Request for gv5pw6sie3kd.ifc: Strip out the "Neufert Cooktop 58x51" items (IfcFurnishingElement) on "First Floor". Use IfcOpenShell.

First a look at what the model holds.

```python
import ifcopenshell
import ifcopenshell.util.element

model = ifcopenshell.open("gv5pw6sie3kd.ifc")
print(model.schema)
storey = next(s for s in model.by_type("IfcBuildingStorey") if s.Name == "First Floor")
furniture = [e for e in ifcopenshell.util.element.get_decomposition(storey) if e.is_a("IfcFurnishingElement")]
seen = {}
for e in furniture:
    element_type = ifcopenshell.util.element.get_type(e)
    name = element_type.Name if element_type not in (None, e) else None
    seen[name] = seen.get(name, 0) + 1
for name, count in sorted(seen.items(), key=str):
    print(count, "x", name)
```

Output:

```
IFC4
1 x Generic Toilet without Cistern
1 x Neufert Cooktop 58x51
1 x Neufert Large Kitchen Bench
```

```python
import ifcopenshell
import ifcopenshell.api.root
import ifcopenshell.util.element

model = ifcopenshell.open("gv5pw6sie3kd.ifc")

storey = next(s for s in model.by_type("IfcBuildingStorey") if s.Name == "First Floor")
furniture = [e for e in ifcopenshell.util.element.get_decomposition(storey) if e.is_a("IfcFurnishingElement")]
targets = [e for e in furniture if (t := ifcopenshell.util.element.get_type(e)) not in (None, e) and t.Name == "Neufert Cooktop 58x51"]

for e in targets:
    ifcopenshell.api.root.remove_product(model, product=e)
print(len(targets), "removed")

model.write("gv5pw6sie3kd_edited.ifc")
```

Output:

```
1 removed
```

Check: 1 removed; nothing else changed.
